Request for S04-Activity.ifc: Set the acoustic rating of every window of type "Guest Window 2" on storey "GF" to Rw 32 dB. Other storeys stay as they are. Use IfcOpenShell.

First a look at what the model holds.

```python
import ifcopenshell
import ifcopenshell.util.element

model = ifcopenshell.open("S04-Activity.ifc")
print(model.schema)
storey = next(s for s in model.by_type("IfcBuildingStorey") if s.Name == "GF")
windows = [e for e in ifcopenshell.util.element.get_decomposition(storey) if e.is_a("IfcWindow")]
seen = {}
for e in windows:
    element_type = ifcopenshell.util.element.get_type(e)
    key = (element_type.Name if element_type != e and element_type else None, ifcopenshell.util.element.get_pset(e, "Pset_WindowCommon", "AcousticRating"))
    seen[key] = seen.get(key, 0) + 1
for (name, value), count in sorted(seen.items(), key=str):
    print(count, "x", name, "|", value)
```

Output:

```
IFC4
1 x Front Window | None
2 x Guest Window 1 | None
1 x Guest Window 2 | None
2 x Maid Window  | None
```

```python
import ifcopenshell
import ifcopenshell.api.pset
import ifcopenshell.util.element

model = ifcopenshell.open("S04-Activity.ifc")

storey = next(s for s in model.by_type("IfcBuildingStorey") if s.Name == "GF")
windows = [e for e in ifcopenshell.util.element.get_decomposition(storey) if e.is_a("IfcWindow")]

count = 0
for e in windows:
    element_type = ifcopenshell.util.element.get_type(e)
    if element_type in (None, e) or element_type.Name != "Guest Window 2":
        continue
    # add_pset returns the element's existing set when there is one.
    pset = ifcopenshell.api.pset.add_pset(model, product=e, name="Pset_WindowCommon")
    ifcopenshell.api.pset.edit_pset(model, pset=pset, properties={"AcousticRating": "Rw 32 dB"})
    count += 1

print(count, "windows updated")

model.write("S04-Activity_edited.ifc")
```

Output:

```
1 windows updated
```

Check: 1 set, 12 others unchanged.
